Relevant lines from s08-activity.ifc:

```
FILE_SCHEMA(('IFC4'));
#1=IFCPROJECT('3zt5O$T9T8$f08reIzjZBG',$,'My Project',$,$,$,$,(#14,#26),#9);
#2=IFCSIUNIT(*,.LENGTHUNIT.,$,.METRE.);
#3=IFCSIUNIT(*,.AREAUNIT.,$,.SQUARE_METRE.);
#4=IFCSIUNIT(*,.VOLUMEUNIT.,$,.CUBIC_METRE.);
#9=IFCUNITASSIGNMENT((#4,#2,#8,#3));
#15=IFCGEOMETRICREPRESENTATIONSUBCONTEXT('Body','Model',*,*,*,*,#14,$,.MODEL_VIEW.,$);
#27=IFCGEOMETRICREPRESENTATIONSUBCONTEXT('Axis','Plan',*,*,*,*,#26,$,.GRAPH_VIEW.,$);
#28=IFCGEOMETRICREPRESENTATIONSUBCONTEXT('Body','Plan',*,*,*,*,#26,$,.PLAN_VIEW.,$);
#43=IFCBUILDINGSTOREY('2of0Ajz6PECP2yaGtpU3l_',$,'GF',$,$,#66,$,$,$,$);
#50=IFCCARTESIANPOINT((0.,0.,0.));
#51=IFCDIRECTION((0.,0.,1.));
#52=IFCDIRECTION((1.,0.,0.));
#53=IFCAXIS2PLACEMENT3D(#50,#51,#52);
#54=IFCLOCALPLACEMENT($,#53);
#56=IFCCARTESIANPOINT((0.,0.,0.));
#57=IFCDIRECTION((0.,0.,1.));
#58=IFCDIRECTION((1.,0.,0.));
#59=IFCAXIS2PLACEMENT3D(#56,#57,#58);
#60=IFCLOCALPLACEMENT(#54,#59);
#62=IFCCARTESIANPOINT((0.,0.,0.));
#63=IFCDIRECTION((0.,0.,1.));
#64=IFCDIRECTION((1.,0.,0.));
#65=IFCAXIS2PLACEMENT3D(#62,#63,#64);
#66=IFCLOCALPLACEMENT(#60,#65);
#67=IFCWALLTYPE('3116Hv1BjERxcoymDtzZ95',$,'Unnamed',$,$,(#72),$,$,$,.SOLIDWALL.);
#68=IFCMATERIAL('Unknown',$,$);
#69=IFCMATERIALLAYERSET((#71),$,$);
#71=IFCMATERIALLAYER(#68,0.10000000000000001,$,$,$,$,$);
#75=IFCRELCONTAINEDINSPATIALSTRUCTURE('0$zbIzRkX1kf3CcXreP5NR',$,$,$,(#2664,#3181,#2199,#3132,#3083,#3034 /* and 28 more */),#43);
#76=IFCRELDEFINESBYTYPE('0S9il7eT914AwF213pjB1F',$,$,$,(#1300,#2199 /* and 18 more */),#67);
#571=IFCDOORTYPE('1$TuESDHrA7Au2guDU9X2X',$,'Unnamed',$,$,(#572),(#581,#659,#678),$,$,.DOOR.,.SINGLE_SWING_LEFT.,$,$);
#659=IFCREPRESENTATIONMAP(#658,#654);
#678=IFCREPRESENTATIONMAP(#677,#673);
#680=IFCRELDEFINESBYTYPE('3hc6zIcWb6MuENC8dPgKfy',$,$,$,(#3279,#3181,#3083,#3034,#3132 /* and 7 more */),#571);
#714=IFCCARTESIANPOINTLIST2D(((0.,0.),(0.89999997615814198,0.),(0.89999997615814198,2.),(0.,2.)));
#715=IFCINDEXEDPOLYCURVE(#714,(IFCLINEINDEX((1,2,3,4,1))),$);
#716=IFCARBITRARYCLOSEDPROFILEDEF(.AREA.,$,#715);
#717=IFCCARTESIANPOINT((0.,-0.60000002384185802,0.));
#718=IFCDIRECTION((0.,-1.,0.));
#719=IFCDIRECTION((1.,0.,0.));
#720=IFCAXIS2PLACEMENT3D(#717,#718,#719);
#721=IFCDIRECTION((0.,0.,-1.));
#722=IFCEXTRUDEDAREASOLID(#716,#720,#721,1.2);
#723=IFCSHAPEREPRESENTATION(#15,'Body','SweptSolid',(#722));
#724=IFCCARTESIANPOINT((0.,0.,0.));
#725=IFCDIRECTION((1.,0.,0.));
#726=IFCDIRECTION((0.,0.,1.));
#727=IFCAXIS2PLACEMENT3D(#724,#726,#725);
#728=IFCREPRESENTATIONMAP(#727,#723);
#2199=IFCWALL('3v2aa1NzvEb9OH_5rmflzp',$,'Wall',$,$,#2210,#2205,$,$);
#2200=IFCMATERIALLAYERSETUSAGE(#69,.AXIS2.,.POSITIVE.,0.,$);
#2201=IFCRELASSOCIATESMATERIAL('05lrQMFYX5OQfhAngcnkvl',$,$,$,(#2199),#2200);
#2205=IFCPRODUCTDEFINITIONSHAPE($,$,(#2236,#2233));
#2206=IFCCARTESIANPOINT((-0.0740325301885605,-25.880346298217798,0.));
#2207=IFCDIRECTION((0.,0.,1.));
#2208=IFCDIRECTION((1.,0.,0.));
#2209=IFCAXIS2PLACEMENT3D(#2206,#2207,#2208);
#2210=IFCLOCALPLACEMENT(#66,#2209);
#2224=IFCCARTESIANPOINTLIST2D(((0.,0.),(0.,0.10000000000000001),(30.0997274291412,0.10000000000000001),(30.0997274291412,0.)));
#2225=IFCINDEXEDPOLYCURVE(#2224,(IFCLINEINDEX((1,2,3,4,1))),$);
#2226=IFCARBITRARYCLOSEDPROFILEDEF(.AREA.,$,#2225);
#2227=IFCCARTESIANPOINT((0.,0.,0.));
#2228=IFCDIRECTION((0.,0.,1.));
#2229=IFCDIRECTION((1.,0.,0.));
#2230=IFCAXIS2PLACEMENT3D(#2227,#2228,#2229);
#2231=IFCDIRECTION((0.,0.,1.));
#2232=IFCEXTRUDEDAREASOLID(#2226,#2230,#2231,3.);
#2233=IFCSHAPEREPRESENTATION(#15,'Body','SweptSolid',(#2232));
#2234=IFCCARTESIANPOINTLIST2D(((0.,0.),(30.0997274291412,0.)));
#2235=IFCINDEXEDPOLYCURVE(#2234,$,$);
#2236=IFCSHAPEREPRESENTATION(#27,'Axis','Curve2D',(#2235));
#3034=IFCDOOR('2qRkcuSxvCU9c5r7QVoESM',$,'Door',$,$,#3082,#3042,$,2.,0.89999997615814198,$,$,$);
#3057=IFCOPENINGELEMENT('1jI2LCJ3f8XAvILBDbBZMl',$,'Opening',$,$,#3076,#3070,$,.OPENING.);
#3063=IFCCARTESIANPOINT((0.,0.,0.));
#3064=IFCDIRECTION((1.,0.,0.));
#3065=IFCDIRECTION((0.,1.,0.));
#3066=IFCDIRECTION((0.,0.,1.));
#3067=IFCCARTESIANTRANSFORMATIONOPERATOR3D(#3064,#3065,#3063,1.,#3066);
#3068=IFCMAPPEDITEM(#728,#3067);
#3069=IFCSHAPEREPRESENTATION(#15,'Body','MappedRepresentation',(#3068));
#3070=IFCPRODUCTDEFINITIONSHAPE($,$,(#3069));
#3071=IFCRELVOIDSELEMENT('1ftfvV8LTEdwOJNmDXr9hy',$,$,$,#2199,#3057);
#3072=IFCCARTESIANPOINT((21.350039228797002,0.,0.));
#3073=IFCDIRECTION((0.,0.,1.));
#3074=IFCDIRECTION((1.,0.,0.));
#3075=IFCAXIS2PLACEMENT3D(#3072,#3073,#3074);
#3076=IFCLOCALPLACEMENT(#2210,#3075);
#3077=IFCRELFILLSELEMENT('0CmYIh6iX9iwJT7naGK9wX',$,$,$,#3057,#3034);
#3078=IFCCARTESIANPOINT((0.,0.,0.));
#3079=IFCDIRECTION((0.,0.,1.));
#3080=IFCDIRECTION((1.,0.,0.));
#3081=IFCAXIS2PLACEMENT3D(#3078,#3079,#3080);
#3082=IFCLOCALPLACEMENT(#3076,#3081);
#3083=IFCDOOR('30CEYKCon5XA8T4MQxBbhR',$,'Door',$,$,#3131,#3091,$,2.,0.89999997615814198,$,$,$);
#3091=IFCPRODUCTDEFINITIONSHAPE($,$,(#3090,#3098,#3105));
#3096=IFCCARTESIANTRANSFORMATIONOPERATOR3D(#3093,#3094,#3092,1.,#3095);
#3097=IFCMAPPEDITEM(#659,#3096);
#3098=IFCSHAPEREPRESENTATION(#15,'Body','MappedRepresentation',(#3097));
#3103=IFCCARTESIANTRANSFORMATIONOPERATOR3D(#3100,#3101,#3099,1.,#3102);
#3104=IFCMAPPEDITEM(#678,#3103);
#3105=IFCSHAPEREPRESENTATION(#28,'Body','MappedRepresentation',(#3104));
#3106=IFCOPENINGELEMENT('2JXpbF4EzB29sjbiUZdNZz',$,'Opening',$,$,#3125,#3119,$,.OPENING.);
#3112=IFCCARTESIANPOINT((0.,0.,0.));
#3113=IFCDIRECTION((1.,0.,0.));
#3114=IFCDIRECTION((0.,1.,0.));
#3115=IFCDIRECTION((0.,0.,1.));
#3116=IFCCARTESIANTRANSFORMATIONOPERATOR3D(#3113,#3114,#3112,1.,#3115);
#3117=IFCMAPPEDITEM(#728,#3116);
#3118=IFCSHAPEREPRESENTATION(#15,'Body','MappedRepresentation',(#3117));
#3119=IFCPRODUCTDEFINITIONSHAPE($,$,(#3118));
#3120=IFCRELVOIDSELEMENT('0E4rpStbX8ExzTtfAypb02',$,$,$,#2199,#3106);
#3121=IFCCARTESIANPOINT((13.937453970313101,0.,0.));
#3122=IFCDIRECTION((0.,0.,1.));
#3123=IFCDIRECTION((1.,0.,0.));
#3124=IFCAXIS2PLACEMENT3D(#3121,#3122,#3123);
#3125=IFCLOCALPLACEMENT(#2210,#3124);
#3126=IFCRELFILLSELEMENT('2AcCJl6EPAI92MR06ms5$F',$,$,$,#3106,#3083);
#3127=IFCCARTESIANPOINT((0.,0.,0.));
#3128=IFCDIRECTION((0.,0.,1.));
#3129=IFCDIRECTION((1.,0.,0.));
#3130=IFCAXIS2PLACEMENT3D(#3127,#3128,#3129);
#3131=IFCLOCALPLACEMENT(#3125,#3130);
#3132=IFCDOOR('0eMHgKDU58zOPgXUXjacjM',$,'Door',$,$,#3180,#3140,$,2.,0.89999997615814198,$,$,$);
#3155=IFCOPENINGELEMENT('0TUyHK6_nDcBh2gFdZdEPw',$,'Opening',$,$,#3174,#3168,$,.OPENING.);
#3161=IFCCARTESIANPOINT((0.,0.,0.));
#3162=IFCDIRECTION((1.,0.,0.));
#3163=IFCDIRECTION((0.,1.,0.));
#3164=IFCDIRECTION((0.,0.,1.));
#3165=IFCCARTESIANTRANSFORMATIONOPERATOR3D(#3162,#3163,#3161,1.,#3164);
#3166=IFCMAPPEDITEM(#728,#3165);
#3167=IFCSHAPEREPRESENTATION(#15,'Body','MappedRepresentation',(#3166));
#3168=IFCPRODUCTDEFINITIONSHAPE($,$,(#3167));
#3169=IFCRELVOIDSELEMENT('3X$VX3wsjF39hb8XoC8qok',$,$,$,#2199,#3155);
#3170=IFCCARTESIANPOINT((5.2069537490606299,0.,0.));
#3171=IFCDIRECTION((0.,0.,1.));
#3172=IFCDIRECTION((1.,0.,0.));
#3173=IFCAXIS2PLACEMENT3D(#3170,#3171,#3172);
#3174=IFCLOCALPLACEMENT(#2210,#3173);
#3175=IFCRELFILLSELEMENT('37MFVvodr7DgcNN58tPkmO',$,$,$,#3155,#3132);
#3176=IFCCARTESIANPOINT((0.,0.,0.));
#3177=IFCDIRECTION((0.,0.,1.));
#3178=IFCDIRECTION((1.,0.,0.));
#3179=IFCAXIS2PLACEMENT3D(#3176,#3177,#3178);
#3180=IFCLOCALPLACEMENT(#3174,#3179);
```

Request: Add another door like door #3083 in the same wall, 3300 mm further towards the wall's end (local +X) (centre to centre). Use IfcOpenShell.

```python
import ifcopenshell
import ifcopenshell.api.feature
import ifcopenshell.api.geometry
import ifcopenshell.api.root
import ifcopenshell.geom
import ifcopenshell.util.element
import ifcopenshell.util.placement
import ifcopenshell.util.shape
import ifcopenshell.util.unit

model = ifcopenshell.open("s08-activity.ifc")
unit_scale = ifcopenshell.util.unit.calculate_unit_scale(model)
settings = ifcopenshell.geom.settings()


def volume(element):
    """Net volume in cubic metres, openings subtracted."""
    shape = ifcopenshell.geom.create_shape(settings, element)
    return ifcopenshell.util.shape.get_volume(shape.geometry)


door = model.by_guid("30CEYKCon5XA8T4MQxBbhR")
opening = door.FillsVoids[0].RelatingOpeningElement
wall = opening.VoidsElements[0].RelatingBuildingElement
before = volume(wall)
shift = ifcopenshell.util.placement.get_local_placement(wall.ObjectPlacement)[:3, 0] * 3.3 / unit_scale

# copy_class copies the void relationship, type, container and properties, but no geometry.
new_opening = ifcopenshell.api.root.copy_class(model, product=opening)
new_opening.Representation = ifcopenshell.util.element.copy_deep(
    model, opening.Representation, exclude=["IfcGeometricRepresentationContext", "IfcRepresentationMap"]
)
new_door = ifcopenshell.api.root.copy_class(model, product=door)
new_door.Representation = ifcopenshell.util.element.copy_deep(
    model, door.Representation, exclude=["IfcGeometricRepresentationContext", "IfcRepresentationMap"]
)
ifcopenshell.api.feature.add_filling(model, opening=new_opening, element=new_door)

for old, new in ((opening, new_opening), (door, new_door)):
    matrix = ifcopenshell.util.placement.get_local_placement(old.ObjectPlacement)
    matrix[:3, 3] += shift
    ifcopenshell.api.geometry.edit_object_placement(model, product=new, matrix=matrix, is_si=False)

after = volume(wall)

print(f"wall volume {before:.3f} -> {after:.3f} m3")

model.write("s08-activity_rev.ifc")
```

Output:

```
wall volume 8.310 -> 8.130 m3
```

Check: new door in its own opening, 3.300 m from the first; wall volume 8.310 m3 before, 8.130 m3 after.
